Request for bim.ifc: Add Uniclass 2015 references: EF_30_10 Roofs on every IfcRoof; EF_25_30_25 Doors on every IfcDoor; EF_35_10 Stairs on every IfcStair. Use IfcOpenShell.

First a look at what the model holds.

```python
import ifcopenshell

model = ifcopenshell.open("bim.ifc")
print(model.schema)
print("classifications:", [c.Name for c in model.by_type("IfcClassification")])
for ifc_class in ("IfcDoor", "IfcRoof", "IfcStair", "IfcWall", "IfcWindow"):
    print(ifc_class, len(model.by_type(ifc_class)))
```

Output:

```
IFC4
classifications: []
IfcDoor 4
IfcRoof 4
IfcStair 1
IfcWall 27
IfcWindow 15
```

```python
import ifcopenshell
import ifcopenshell.api.classification

model = ifcopenshell.open("bim.ifc")

system = ifcopenshell.api.classification.add_classification(model, classification="Uniclass 2015")

codes = {
    "IfcRoof": ("EF_30_10", "Roofs"),
    "IfcDoor": ("EF_25_30_25", "Doors"),
    "IfcStair": ("EF_35_10", "Stairs"),
}
for ifc_class, (code, name) in codes.items():
    products = model.by_type(ifc_class)
    ifcopenshell.api.classification.add_reference(
        model, products=products, classification=system, identification=code, name=name
    )
    print(code, len(products))

model.write("bim-out.ifc")
```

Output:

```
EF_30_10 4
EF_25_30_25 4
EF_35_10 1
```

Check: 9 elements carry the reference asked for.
